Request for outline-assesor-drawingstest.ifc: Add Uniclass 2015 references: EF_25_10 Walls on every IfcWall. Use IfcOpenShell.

First a look at what the model holds.

```python
import ifcopenshell

model = ifcopenshell.open("outline-assesor-drawingstest.ifc")
print(model.schema)
print("classifications:", [c.Name for c in model.by_type("IfcClassification")])
for ifc_class in ("IfcDoor", "IfcRoof", "IfcStair", "IfcWall", "IfcWindow"):
    print(ifc_class, len(model.by_type(ifc_class)))
```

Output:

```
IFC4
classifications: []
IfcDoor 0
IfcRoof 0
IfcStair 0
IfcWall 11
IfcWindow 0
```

```python
import ifcopenshell
import ifcopenshell.api.classification

model = ifcopenshell.open("outline-assesor-drawingstest.ifc")

system = ifcopenshell.api.classification.add_classification(model, classification="Uniclass 2015")

codes = {
    "IfcWall": ("EF_25_10", "Walls"),
}
for ifc_class, (code, name) in codes.items():
    products = model.by_type(ifc_class)
    ifcopenshell.api.classification.add_reference(
        model, products=products, classification=system, identification=code, name=name
    )
    print(code, len(products))

model.write("outline-assesor-drawingstest_edited.ifc")
```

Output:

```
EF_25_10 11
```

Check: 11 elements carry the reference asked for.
